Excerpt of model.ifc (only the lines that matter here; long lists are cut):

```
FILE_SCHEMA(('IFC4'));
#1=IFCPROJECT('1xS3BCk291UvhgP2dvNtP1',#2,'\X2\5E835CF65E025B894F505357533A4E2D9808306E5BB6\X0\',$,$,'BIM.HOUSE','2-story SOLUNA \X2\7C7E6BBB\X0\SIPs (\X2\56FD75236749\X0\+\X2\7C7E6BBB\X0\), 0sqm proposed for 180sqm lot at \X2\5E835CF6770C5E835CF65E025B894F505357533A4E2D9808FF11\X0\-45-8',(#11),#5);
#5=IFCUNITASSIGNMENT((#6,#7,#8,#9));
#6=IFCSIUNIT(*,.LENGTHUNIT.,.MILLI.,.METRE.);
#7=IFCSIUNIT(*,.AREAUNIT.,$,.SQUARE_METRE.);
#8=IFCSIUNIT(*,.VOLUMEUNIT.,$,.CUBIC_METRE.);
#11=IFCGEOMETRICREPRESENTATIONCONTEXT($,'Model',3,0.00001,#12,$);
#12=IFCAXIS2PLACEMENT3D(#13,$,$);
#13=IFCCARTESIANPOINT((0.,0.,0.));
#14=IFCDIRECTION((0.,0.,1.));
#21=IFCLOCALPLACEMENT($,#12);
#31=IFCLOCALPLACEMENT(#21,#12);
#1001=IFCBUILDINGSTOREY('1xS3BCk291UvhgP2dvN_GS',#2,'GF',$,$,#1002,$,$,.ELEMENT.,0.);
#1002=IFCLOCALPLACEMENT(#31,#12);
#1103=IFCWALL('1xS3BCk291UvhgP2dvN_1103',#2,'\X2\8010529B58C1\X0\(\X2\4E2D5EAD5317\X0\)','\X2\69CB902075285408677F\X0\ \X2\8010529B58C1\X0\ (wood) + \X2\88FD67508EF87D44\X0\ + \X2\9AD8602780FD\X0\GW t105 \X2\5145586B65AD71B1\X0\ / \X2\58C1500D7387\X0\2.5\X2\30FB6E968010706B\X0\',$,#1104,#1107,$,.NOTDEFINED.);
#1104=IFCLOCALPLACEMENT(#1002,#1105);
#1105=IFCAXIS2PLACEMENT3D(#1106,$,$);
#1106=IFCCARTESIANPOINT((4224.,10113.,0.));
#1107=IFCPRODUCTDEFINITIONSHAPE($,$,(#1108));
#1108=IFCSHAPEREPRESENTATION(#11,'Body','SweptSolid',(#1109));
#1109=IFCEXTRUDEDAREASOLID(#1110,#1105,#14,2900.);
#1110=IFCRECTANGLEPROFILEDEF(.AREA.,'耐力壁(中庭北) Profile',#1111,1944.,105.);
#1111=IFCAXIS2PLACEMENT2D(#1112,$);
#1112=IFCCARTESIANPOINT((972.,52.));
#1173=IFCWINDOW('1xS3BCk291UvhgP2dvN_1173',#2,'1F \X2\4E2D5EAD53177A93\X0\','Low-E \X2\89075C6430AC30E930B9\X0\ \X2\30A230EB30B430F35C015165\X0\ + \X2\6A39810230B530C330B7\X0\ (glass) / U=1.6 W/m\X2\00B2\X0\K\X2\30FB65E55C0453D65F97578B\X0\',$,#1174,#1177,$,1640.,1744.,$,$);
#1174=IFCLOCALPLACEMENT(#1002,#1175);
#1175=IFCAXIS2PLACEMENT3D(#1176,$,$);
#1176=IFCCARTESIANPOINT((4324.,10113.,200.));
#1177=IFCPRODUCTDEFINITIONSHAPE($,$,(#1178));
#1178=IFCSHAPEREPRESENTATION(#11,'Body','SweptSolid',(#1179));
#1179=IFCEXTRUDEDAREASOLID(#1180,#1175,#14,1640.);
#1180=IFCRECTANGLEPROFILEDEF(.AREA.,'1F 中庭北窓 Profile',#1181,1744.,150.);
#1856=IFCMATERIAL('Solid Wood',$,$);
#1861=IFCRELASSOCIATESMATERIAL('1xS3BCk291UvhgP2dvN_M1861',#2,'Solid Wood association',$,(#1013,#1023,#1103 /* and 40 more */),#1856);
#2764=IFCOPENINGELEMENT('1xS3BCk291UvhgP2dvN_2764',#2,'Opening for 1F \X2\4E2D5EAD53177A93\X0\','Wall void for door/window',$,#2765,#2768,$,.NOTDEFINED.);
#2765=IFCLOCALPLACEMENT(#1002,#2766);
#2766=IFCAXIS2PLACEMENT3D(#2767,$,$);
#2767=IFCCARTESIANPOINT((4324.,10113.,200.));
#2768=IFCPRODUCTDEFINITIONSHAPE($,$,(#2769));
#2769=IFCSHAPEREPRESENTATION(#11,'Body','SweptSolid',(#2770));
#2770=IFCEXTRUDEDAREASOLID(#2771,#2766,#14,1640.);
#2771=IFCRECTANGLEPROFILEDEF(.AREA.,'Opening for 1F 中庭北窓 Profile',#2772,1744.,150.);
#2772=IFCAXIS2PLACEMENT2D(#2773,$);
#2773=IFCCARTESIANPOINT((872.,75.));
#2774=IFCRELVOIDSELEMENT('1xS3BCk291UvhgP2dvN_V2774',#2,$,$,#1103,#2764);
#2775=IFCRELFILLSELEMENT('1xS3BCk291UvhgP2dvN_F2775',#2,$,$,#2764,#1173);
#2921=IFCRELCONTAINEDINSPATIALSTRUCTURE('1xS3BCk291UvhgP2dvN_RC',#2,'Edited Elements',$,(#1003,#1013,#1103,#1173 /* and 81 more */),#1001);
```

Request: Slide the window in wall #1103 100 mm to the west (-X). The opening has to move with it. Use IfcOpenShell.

```python
import ifcopenshell
import ifcopenshell.api.geometry
import ifcopenshell.util.placement

model = ifcopenshell.open("model.ifc")

window = model.by_id(1173)
opening = window.FillsVoids[0].RelatingOpeningElement
wall = opening.VoidsElements[0].RelatingBuildingElement

wall_matrix = ifcopenshell.util.placement.get_local_placement(wall.ObjectPlacement)
shift = wall_matrix[:3, 0] * -100.0
before = ifcopenshell.util.placement.get_local_placement(window.ObjectPlacement)[:3, 3].copy()

# The window is not placed relative to its opening, so move both.
for product in (opening, window):
    matrix = ifcopenshell.util.placement.get_local_placement(product.ObjectPlacement)
    matrix[:3, 3] += shift
    ifcopenshell.api.geometry.edit_object_placement(model, product=product, matrix=matrix, is_si=False)

after = ifcopenshell.util.placement.get_local_placement(window.ObjectPlacement)[:3, 3]
print("window moved by", (after - before).round(3) + 0.0)

model.write("model-out.ifc")
```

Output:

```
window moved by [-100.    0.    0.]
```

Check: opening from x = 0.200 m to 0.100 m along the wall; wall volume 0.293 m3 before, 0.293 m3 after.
